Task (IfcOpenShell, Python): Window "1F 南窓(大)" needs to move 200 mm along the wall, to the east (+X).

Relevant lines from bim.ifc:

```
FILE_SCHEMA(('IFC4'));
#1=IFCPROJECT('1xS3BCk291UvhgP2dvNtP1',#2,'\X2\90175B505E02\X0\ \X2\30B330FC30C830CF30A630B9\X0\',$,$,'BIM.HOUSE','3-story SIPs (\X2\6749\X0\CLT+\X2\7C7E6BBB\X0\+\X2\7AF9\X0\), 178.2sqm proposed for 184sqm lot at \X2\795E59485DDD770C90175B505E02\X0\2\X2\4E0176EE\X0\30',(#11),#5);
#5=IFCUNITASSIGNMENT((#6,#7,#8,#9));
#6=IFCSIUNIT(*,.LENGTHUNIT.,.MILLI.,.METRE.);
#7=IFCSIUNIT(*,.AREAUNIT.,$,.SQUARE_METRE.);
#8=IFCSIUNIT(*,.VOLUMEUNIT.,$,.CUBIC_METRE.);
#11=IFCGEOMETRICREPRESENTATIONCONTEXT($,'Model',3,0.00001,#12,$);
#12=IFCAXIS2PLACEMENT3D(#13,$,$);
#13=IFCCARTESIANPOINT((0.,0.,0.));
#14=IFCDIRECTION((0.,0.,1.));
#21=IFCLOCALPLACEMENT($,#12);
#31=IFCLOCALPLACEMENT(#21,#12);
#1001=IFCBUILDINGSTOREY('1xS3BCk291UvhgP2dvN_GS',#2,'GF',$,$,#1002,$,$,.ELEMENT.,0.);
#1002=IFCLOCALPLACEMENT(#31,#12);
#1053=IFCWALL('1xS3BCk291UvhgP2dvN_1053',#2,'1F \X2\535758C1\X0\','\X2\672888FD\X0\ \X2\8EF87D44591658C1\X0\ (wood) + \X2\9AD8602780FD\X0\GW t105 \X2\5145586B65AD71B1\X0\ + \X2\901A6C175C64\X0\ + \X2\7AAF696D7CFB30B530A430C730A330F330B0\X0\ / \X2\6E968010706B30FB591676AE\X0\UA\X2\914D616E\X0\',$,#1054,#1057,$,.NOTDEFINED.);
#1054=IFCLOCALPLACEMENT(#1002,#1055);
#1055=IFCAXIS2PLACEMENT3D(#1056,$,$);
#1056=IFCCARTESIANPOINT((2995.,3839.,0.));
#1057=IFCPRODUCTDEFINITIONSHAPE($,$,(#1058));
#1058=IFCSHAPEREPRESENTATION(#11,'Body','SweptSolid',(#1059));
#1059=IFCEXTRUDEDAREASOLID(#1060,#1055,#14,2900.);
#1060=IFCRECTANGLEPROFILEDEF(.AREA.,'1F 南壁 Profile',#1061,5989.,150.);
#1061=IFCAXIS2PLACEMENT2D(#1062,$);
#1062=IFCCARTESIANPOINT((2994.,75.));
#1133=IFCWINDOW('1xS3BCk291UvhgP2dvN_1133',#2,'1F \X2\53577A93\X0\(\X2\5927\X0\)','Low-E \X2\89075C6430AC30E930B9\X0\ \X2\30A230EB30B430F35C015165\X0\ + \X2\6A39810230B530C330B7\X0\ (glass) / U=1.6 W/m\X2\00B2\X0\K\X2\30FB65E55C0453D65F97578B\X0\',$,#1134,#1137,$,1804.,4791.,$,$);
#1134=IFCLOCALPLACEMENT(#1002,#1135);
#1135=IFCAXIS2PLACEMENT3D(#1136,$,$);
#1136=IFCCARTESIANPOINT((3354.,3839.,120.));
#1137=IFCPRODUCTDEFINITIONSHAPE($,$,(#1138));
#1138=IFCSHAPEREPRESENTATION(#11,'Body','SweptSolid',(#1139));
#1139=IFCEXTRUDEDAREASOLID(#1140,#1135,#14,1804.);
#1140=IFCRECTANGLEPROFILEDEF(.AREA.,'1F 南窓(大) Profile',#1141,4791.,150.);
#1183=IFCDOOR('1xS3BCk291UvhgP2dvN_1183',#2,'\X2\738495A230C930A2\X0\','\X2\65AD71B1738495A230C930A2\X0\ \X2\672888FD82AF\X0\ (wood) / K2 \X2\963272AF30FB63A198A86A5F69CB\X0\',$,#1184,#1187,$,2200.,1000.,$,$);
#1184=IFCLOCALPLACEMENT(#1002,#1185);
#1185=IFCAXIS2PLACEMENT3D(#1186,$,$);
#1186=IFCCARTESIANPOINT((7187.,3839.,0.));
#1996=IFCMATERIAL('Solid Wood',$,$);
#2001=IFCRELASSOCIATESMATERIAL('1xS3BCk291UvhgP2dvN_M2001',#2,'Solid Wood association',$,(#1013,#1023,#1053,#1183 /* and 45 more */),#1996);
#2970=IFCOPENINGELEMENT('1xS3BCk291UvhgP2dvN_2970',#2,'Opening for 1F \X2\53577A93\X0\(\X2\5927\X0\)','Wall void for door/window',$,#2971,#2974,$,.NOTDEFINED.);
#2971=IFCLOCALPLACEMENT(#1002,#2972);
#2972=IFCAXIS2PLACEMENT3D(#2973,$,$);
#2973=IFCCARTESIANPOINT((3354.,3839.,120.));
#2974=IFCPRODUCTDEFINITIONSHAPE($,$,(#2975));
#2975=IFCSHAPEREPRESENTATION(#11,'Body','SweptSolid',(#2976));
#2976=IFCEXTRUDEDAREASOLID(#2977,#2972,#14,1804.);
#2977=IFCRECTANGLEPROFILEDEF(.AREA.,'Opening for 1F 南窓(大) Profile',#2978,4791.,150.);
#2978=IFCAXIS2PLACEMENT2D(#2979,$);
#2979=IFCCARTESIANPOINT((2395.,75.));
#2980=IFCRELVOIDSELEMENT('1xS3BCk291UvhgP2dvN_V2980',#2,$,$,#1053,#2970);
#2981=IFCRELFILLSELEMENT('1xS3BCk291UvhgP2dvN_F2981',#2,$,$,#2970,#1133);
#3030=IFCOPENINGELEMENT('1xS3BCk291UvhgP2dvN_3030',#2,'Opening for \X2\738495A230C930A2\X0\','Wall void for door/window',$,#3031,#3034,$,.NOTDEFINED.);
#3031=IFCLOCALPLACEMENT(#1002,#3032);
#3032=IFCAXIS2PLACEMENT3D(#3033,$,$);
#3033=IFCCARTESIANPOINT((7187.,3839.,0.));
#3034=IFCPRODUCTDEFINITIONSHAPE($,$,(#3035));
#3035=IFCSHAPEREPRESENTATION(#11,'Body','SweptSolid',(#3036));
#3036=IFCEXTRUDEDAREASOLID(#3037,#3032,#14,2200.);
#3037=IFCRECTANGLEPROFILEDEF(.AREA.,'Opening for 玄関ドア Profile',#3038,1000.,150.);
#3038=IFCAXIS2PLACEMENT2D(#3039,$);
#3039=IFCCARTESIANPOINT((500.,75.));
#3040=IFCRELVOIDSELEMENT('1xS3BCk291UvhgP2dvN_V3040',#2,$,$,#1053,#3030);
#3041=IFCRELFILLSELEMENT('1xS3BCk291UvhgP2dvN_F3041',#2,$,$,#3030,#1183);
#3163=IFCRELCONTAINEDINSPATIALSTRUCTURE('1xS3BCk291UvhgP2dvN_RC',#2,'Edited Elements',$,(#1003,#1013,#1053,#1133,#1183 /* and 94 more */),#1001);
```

```python
import ifcopenshell
import ifcopenshell.api.geometry
import ifcopenshell.util.placement

model = ifcopenshell.open("bim.ifc")

window = model.by_guid("1xS3BCk291UvhgP2dvN_1133")
opening = window.FillsVoids[0].RelatingOpeningElement
wall = opening.VoidsElements[0].RelatingBuildingElement

wall_matrix = ifcopenshell.util.placement.get_local_placement(wall.ObjectPlacement)
shift = wall_matrix[:3, 0] * 200.0
before = ifcopenshell.util.placement.get_local_placement(window.ObjectPlacement)[:3, 3].copy()

# The window is not placed relative to its opening, so move both.
for product in (opening, window):
    matrix = ifcopenshell.util.placement.get_local_placement(product.ObjectPlacement)
    matrix[:3, 3] += shift
    ifcopenshell.api.geometry.edit_object_placement(model, product=product, matrix=matrix, is_si=False)

after = ifcopenshell.util.placement.get_local_placement(window.ObjectPlacement)[:3, 3]
print("window moved by", (after - before).round(3) + 0.0)

model.write("bim_edited.ifc")
```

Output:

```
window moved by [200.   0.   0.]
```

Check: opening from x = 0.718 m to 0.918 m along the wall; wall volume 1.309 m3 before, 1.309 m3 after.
